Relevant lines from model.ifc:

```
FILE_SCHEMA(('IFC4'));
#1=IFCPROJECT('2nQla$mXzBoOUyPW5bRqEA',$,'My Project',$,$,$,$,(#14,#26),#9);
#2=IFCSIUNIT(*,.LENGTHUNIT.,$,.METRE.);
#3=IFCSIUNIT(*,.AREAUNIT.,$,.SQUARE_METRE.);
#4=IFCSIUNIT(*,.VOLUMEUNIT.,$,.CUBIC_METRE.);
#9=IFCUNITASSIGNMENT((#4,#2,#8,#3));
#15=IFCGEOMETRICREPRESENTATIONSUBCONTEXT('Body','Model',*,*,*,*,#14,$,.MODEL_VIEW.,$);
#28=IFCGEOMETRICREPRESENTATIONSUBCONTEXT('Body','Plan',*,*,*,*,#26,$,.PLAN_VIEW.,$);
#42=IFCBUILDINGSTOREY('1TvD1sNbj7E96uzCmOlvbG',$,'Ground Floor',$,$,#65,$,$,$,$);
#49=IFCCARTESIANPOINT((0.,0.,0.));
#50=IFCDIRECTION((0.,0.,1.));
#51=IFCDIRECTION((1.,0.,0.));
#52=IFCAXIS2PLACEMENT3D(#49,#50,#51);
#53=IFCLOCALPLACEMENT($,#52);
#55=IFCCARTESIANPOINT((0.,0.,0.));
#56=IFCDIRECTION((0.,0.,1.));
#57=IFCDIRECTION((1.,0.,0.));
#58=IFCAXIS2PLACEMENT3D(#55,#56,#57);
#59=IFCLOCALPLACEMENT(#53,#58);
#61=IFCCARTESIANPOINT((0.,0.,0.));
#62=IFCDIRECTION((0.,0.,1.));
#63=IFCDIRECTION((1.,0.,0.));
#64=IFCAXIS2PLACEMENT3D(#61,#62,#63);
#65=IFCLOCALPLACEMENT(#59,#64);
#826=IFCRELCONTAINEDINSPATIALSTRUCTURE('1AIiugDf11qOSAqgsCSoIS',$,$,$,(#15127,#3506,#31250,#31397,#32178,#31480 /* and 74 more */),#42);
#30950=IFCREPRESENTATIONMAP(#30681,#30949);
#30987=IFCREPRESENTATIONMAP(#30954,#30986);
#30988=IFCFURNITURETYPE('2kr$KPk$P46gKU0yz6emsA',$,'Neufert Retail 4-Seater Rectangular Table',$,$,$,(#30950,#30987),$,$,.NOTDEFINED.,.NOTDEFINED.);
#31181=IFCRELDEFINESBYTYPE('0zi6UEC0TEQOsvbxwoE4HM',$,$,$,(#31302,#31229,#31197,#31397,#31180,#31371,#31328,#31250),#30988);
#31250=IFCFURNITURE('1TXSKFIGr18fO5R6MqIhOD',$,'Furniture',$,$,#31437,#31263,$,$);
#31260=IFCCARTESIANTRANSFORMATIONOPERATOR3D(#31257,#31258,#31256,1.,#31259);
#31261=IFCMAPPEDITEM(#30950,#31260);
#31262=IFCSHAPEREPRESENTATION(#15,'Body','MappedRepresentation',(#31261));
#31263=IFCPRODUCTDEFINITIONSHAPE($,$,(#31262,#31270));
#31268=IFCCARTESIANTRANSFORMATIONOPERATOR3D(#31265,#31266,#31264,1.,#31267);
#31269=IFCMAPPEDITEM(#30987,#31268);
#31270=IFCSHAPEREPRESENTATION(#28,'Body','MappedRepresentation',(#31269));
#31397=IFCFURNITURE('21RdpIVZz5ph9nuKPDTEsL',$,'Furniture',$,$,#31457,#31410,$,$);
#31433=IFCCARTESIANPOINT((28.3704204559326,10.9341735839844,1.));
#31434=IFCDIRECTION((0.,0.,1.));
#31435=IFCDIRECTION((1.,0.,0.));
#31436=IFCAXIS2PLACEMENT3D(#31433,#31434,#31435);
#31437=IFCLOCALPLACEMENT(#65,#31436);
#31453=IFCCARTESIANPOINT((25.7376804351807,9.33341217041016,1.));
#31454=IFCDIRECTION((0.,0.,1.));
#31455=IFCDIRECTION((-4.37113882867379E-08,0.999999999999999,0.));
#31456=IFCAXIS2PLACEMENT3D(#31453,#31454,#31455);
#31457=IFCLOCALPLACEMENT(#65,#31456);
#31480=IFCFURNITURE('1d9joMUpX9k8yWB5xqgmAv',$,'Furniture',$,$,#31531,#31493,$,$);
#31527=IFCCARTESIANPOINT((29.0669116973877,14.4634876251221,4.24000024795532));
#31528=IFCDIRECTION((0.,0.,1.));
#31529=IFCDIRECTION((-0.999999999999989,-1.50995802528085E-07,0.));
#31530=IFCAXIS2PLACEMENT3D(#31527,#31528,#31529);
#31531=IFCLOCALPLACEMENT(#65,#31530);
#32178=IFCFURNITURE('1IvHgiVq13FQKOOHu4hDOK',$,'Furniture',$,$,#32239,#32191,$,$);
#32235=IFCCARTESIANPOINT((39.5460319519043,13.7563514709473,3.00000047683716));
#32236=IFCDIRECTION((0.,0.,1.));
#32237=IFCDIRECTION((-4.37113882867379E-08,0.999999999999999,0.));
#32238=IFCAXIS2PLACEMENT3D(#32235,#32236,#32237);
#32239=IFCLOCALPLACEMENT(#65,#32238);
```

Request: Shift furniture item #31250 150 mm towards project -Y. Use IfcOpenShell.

```python
import ifcopenshell
import ifcopenshell.api.geometry
import ifcopenshell.util.placement

model = ifcopenshell.open("model.ifc")

item = model.by_guid("1TXSKFIGr18fO5R6MqIhOD")
matrix = ifcopenshell.util.placement.get_local_placement(item.ObjectPlacement)
matrix[1, 3] -= 0.15
ifcopenshell.api.geometry.edit_object_placement(model, product=item, matrix=matrix, is_si=False)

print(ifcopenshell.util.placement.get_local_placement(item.ObjectPlacement).round(3) + 0.0)

model.write("model_edited.ifc")
```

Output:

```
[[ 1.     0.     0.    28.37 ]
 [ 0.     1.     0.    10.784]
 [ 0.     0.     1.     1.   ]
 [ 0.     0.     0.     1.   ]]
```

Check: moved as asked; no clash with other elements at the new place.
